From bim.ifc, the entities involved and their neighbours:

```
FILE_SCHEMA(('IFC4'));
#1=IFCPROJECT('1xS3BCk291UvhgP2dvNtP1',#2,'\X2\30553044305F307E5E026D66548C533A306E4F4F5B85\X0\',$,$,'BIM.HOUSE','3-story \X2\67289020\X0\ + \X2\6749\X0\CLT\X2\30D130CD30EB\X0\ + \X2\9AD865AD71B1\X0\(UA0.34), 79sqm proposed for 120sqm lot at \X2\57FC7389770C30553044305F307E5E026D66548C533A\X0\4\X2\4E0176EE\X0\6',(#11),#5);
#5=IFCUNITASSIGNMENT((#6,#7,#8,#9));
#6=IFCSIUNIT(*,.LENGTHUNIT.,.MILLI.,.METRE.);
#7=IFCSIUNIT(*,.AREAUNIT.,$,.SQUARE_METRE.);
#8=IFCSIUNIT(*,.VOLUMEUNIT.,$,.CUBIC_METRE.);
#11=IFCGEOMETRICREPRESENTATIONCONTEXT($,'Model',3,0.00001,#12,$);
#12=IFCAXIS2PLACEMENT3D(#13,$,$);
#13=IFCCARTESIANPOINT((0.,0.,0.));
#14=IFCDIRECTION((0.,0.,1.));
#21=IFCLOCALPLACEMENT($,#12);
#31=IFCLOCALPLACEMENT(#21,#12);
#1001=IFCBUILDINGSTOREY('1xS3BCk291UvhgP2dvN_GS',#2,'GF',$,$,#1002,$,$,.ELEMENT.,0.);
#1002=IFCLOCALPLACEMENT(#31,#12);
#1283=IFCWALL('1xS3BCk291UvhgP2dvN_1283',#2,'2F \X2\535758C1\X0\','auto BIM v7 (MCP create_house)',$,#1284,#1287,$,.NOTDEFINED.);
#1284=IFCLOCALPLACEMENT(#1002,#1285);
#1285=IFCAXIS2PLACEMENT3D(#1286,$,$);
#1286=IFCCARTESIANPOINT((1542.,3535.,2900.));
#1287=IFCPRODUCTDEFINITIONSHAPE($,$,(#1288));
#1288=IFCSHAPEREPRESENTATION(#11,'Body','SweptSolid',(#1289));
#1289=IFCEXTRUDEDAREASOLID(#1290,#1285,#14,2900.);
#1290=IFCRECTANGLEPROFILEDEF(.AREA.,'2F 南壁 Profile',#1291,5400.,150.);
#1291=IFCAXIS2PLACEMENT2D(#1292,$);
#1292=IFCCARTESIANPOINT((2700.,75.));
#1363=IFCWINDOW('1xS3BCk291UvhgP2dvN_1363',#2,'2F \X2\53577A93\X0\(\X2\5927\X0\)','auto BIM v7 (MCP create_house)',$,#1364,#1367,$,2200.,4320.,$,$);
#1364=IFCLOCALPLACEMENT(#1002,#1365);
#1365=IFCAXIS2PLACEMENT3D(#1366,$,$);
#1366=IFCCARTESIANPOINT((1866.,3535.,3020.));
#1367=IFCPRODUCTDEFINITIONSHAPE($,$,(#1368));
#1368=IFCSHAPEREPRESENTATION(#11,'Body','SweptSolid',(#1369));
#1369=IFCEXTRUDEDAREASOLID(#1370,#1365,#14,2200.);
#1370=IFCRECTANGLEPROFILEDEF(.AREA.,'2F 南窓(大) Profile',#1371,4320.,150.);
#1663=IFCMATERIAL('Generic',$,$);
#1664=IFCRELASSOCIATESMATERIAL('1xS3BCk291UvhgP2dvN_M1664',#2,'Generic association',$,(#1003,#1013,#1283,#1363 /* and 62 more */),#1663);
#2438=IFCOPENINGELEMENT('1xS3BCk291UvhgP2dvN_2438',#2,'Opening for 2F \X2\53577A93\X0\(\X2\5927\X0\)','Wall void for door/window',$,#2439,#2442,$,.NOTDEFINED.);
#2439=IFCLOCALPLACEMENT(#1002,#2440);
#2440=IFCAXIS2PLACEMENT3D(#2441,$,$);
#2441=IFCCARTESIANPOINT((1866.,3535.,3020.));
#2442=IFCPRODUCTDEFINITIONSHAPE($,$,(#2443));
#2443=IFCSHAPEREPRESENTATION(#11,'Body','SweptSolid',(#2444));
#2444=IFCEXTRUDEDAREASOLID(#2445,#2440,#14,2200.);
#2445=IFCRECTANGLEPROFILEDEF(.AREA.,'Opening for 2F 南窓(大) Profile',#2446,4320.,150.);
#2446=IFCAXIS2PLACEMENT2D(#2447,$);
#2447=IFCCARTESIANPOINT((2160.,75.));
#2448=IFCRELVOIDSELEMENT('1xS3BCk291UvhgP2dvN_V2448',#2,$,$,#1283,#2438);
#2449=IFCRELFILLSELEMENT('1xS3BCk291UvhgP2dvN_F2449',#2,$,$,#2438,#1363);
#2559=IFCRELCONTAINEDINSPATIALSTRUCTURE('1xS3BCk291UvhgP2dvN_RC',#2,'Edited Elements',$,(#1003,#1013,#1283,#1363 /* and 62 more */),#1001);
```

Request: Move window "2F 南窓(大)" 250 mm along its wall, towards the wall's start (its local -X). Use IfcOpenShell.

```python
import ifcopenshell
import ifcopenshell.api.geometry
import ifcopenshell.util.placement
import ifcopenshell.util.unit

model = ifcopenshell.open("bim.ifc")
unit_scale = ifcopenshell.util.unit.calculate_unit_scale(model)

window = model.by_guid("1xS3BCk291UvhgP2dvN_1363")
opening = window.FillsVoids[0].RelatingOpeningElement
wall = opening.VoidsElements[0].RelatingBuildingElement

wall_matrix = ifcopenshell.util.placement.get_local_placement(wall.ObjectPlacement)
shift = wall_matrix[:3, 0] * -0.25 / unit_scale
before = ifcopenshell.util.placement.get_local_placement(window.ObjectPlacement)[:3, 3].copy()

# The window is not placed relative to its opening, so move both.
for product in (opening, window):
    matrix = ifcopenshell.util.placement.get_local_placement(product.ObjectPlacement)
    matrix[:3, 3] += shift
    ifcopenshell.api.geometry.edit_object_placement(model, product=product, matrix=matrix, is_si=False)

after = ifcopenshell.util.placement.get_local_placement(window.ObjectPlacement)[:3, 3]
print("window moved by", (after - before).round(3) + 0.0)

model.write("bim_rev.ifc")
```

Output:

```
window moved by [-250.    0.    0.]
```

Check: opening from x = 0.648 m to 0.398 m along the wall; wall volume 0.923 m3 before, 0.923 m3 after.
